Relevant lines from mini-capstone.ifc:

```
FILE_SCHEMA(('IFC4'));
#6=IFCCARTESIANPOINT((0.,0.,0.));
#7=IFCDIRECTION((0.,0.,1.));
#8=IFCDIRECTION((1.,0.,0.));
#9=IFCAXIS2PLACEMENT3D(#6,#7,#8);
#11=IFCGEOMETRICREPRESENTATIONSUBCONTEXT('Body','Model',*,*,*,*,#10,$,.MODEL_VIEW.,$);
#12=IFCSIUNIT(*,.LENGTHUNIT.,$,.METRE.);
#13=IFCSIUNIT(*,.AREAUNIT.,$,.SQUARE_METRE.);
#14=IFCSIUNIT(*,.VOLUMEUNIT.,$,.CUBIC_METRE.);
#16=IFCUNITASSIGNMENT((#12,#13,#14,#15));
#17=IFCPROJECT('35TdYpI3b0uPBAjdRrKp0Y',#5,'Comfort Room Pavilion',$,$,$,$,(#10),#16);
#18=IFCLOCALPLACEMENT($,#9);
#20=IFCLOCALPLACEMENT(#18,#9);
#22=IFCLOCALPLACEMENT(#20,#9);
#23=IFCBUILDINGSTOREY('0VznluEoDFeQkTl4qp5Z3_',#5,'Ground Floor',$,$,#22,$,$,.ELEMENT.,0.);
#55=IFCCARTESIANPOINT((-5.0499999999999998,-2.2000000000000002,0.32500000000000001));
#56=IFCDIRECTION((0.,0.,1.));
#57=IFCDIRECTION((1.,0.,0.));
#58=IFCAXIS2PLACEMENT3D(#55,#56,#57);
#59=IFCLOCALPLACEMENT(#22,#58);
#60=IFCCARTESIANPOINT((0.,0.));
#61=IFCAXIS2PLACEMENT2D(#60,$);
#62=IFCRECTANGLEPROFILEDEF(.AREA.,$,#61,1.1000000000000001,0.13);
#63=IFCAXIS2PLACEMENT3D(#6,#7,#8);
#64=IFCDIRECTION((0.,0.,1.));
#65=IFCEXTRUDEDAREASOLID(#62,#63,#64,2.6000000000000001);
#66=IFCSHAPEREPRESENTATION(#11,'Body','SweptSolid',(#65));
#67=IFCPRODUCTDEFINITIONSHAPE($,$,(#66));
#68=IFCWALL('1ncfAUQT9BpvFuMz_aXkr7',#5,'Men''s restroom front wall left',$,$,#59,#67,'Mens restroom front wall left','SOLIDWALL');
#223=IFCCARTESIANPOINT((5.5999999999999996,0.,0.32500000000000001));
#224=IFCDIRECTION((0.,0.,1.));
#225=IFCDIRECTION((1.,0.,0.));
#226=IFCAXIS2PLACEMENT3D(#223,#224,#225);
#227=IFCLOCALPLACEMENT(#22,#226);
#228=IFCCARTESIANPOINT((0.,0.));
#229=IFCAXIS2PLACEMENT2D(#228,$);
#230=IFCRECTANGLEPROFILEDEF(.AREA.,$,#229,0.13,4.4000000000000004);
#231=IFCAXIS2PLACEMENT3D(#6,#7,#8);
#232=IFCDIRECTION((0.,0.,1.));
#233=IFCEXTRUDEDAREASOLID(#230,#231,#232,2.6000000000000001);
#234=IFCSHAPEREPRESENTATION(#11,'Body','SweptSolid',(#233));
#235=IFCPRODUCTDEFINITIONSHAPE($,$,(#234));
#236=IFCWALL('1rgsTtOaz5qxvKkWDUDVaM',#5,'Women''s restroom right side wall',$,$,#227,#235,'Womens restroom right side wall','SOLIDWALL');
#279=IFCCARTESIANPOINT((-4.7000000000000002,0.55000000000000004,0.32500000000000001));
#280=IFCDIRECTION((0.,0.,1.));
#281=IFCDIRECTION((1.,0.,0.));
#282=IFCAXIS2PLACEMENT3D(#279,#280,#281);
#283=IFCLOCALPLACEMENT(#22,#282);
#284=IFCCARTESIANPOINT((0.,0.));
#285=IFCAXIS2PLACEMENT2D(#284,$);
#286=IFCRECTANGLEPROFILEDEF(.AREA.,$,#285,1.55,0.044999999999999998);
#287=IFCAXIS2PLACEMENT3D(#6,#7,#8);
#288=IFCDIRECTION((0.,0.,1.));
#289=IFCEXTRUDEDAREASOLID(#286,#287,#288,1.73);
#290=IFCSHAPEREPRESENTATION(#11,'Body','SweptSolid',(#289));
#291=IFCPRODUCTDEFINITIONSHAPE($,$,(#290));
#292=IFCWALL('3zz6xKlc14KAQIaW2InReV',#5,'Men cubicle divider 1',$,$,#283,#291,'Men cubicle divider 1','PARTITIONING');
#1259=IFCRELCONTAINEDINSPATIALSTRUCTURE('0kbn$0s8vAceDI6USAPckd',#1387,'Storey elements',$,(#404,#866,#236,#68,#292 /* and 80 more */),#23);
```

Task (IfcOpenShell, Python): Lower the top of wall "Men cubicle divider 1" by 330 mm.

```python
import ifcopenshell
import ifcopenshell.geom
import ifcopenshell.util.representation
import ifcopenshell.util.shape

model = ifcopenshell.open("mini-capstone.ifc")
settings = ifcopenshell.geom.settings()


def volume(element):
    """Net volume in cubic metres, openings subtracted."""
    shape = ifcopenshell.geom.create_shape(settings, element)
    return ifcopenshell.util.shape.get_volume(shape.geometry)


wall = model.by_guid("3zz6xKlc14KAQIaW2InReV")
before = volume(wall)

body = ifcopenshell.util.representation.get_representation(wall, "Model", "Body")
solid = body.Items[0]
old_height = solid.Depth
solid.Depth -= 0.33
after = volume(wall)

print(f"height {old_height:g} -> {solid.Depth:g}, volume {before:.3f} -> {after:.3f} m3")

model.write("mini-capstone-out.ifc")
```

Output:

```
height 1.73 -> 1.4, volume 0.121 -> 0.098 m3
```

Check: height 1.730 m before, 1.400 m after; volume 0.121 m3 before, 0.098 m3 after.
